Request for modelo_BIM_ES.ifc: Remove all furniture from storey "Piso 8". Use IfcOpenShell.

First a look at what the model holds.

```python
import ifcopenshell
import ifcopenshell.util.element

model = ifcopenshell.open("modelo_BIM_ES.ifc")
print(model.schema)
storey = next(s for s in model.by_type("IfcBuildingStorey") if s.Name == "Piso 8")
furniture = [e for e in ifcopenshell.util.element.get_decomposition(storey) if e.is_a("IfcFurnishingElement")]
seen = {}
for e in furniture:
    element_type = ifcopenshell.util.element.get_type(e)
    name = element_type.Name if element_type not in (None, e) else None
    seen[name] = seen.get(name, 0) + 1
for name, count in sorted(seen.items(), key=str):
    print(count, "x", name)
```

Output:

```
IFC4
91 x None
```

```python
import ifcopenshell
import ifcopenshell.api.root
import ifcopenshell.util.element

model = ifcopenshell.open("modelo_BIM_ES.ifc")

storey = next(s for s in model.by_type("IfcBuildingStorey") if s.Name == "Piso 8")
furniture = [e for e in ifcopenshell.util.element.get_decomposition(storey) if e.is_a("IfcFurnishingElement")]

for e in furniture:
    ifcopenshell.api.root.remove_product(model, product=e)
print(len(furniture), "removed")

model.write("modelo_BIM_ES_edited.ifc")
```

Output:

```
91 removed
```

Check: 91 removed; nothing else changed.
